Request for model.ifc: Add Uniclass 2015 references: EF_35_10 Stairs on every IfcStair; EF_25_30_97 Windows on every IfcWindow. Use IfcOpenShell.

First a look at what the model holds.

```python
import ifcopenshell

model = ifcopenshell.open("model.ifc")
print(model.schema)
print("classifications:", [c.Name for c in model.by_type("IfcClassification")])
for ifc_class in ("IfcDoor", "IfcRoof", "IfcStair", "IfcWall", "IfcWindow"):
    print(ifc_class, len(model.by_type(ifc_class)))
```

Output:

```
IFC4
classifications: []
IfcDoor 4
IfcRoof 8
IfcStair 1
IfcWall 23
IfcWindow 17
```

```python
import ifcopenshell
import ifcopenshell.api.classification

model = ifcopenshell.open("model.ifc")

system = ifcopenshell.api.classification.add_classification(model, classification="Uniclass 2015")

codes = {
    "IfcStair": ("EF_35_10", "Stairs"),
    "IfcWindow": ("EF_25_30_97", "Windows"),
}
for ifc_class, (code, name) in codes.items():
    products = model.by_type(ifc_class)
    ifcopenshell.api.classification.add_reference(
        model, products=products, classification=system, identification=code, name=name
    )
    print(code, len(products))

model.write("model_v2.ifc")
```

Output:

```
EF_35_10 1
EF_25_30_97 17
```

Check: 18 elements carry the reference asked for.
